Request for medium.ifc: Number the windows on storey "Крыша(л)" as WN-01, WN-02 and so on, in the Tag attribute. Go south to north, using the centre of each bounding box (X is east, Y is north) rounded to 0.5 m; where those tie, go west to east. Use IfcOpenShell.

First a look at what the model holds.

```python
import ifcopenshell
import ifcopenshell.util.element
import ifcopenshell.util.placement

model = ifcopenshell.open("medium.ifc")
print(model.schema)
storey = next(s for s in model.by_type("IfcBuildingStorey") if s.Name == "Крыша(л)")
windows = [e for e in ifcopenshell.util.element.get_decomposition(storey) if e.is_a("IfcWindow")]
for e in sorted(windows, key=lambda e: e.id()):
    origin = ifcopenshell.util.placement.get_local_placement(e.ObjectPlacement)[:3, 3]
    print(e.id(), e.Tag, e.Name, origin.round(2) + 0.0, sep=" | ")
```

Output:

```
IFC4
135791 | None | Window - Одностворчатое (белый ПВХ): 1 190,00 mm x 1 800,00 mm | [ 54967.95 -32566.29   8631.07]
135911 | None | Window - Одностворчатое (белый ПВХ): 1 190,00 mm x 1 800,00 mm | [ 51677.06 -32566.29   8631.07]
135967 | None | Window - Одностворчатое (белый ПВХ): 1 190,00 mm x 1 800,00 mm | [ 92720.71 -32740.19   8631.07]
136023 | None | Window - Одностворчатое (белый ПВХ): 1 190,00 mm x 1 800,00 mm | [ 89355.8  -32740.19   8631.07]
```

```python
import ifcopenshell
import ifcopenshell.geom
import ifcopenshell.util.element
import ifcopenshell.util.shape

model = ifcopenshell.open("medium.ifc")
settings = ifcopenshell.geom.settings()
settings.set("use-world-coords", True)


def centre(element):
    shape = ifcopenshell.geom.create_shape(settings, element)
    return ifcopenshell.util.shape.get_bbox_centroid(shape.geometry)


storey = next(s for s in model.by_type("IfcBuildingStorey") if s.Name == "Крыша(л)")
windows = [e for e in ifcopenshell.util.element.get_decomposition(storey) if e.is_a("IfcWindow")]

# Insertion points can sit at a corner or the storey origin, so sort by the geometry (in metres).
centres = {e: centre(e) for e in windows}
windows.sort(key=lambda e: (round(centres[e][1] / 0.5), centres[e][0]))

for i, e in enumerate(windows, start=1):
    number = f"WN-{i:02d}"
    e.Tag = number
    print(e.id(), number)

model.write("medium-out.ifc")
```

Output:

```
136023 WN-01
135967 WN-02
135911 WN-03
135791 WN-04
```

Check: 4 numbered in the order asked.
